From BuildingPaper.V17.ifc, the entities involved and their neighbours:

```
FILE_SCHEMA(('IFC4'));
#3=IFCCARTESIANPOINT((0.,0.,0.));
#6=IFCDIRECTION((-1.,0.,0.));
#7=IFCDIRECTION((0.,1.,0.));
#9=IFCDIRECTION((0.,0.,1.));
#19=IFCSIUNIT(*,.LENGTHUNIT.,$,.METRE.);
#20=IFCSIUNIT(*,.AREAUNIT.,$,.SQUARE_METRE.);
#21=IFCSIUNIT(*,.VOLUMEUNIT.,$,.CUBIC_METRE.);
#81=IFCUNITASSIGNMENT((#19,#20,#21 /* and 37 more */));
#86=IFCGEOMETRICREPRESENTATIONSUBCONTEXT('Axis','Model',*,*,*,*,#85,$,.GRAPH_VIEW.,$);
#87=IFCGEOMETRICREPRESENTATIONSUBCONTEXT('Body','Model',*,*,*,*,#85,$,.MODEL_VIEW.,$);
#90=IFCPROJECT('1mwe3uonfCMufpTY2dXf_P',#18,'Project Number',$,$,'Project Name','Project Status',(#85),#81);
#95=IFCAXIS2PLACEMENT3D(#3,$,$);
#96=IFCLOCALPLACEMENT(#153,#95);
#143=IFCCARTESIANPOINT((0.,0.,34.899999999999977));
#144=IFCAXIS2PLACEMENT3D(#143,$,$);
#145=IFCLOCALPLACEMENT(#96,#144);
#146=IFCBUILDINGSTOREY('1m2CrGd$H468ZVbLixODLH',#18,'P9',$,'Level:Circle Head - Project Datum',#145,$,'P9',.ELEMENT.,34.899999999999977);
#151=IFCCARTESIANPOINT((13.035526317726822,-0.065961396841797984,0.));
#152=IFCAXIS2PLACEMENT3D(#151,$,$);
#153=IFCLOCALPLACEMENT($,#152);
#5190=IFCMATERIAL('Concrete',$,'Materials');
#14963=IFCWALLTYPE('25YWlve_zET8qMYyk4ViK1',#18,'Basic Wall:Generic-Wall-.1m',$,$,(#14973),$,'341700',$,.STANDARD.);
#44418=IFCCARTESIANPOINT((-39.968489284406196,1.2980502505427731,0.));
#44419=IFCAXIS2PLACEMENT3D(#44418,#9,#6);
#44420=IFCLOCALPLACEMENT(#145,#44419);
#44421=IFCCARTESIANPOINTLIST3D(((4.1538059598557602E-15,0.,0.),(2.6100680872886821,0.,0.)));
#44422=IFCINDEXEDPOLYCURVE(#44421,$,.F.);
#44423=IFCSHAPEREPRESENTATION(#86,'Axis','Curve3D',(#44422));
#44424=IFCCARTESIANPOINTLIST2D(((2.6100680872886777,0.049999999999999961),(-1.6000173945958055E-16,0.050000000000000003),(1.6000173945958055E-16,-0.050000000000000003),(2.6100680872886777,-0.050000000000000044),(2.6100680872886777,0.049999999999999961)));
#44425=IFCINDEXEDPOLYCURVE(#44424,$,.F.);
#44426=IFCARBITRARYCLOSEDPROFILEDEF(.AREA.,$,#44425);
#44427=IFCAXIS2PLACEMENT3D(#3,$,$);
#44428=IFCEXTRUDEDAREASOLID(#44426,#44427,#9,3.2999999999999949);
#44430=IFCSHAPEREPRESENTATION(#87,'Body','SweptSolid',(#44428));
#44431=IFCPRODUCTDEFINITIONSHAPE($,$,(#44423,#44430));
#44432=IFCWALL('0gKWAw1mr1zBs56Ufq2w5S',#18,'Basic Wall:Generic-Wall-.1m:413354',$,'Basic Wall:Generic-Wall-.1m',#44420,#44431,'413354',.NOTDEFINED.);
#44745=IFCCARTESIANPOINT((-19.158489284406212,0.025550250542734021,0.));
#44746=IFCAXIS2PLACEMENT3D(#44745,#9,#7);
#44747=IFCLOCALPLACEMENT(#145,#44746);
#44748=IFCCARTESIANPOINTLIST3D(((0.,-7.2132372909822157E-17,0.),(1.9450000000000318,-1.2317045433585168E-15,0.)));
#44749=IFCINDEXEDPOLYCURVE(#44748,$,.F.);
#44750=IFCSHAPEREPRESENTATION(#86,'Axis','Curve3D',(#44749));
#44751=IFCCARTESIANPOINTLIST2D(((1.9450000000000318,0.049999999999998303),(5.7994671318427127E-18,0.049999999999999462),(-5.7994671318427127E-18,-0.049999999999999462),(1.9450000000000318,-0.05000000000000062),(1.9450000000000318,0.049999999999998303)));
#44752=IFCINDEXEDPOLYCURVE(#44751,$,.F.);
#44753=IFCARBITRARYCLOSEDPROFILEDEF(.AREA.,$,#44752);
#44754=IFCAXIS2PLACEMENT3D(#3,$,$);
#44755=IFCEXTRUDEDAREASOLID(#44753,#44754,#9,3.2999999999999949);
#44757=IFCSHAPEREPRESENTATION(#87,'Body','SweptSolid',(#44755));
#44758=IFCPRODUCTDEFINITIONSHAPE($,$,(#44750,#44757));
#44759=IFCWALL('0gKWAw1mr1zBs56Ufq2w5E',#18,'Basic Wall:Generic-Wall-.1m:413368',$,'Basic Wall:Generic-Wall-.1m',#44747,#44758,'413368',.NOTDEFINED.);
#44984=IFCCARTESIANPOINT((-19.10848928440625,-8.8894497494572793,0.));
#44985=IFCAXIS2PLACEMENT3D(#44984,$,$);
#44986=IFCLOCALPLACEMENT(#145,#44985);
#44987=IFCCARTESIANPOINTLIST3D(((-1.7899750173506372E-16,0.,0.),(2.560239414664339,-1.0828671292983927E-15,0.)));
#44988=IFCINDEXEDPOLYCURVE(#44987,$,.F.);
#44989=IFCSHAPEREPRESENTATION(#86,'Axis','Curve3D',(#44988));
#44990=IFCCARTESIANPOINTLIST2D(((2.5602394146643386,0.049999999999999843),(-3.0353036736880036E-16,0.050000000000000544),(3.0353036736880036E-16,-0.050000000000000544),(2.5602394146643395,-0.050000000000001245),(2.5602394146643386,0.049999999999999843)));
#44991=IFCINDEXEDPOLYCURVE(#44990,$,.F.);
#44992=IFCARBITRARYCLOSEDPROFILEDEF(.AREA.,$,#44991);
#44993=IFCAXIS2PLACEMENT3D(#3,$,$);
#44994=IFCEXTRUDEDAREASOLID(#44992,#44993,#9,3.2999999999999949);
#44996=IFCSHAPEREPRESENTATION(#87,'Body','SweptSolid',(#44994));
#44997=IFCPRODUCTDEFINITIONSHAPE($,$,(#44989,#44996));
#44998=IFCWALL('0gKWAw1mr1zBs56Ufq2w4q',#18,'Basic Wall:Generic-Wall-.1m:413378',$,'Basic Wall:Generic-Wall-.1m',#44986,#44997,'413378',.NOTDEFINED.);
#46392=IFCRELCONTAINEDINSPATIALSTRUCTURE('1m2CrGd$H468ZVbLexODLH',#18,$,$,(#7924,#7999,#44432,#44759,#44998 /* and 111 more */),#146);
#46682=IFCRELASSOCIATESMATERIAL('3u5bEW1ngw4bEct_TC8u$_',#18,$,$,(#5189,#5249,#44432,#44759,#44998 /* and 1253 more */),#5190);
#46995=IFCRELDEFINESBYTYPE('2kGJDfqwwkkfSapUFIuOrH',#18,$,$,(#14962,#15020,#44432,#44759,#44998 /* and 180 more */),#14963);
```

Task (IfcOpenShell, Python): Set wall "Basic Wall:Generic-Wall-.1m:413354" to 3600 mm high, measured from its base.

```python
import ifcopenshell
import ifcopenshell.geom
import ifcopenshell.util.representation
import ifcopenshell.util.shape
import ifcopenshell.util.unit

model = ifcopenshell.open("BuildingPaper.V17.ifc")
unit_scale = ifcopenshell.util.unit.calculate_unit_scale(model)
settings = ifcopenshell.geom.settings()


def volume(element):
    """Net volume in cubic metres, openings subtracted."""
    shape = ifcopenshell.geom.create_shape(settings, element)
    return ifcopenshell.util.shape.get_volume(shape.geometry)


wall = model.by_guid("0gKWAw1mr1zBs56Ufq2w5S")
before = volume(wall)

body = ifcopenshell.util.representation.get_representation(wall, "Model", "Body")
solid = body.Items[0]
old_height = solid.Depth
solid.Depth = 3.6 / unit_scale
after = volume(wall)

print(f"height {old_height:g} -> {solid.Depth:g}, volume {before:.3f} -> {after:.3f} m3")

model.write("BuildingPaper.V17_updated.ifc")
```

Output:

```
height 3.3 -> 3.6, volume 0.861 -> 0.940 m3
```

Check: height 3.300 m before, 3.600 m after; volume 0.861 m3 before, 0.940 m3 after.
